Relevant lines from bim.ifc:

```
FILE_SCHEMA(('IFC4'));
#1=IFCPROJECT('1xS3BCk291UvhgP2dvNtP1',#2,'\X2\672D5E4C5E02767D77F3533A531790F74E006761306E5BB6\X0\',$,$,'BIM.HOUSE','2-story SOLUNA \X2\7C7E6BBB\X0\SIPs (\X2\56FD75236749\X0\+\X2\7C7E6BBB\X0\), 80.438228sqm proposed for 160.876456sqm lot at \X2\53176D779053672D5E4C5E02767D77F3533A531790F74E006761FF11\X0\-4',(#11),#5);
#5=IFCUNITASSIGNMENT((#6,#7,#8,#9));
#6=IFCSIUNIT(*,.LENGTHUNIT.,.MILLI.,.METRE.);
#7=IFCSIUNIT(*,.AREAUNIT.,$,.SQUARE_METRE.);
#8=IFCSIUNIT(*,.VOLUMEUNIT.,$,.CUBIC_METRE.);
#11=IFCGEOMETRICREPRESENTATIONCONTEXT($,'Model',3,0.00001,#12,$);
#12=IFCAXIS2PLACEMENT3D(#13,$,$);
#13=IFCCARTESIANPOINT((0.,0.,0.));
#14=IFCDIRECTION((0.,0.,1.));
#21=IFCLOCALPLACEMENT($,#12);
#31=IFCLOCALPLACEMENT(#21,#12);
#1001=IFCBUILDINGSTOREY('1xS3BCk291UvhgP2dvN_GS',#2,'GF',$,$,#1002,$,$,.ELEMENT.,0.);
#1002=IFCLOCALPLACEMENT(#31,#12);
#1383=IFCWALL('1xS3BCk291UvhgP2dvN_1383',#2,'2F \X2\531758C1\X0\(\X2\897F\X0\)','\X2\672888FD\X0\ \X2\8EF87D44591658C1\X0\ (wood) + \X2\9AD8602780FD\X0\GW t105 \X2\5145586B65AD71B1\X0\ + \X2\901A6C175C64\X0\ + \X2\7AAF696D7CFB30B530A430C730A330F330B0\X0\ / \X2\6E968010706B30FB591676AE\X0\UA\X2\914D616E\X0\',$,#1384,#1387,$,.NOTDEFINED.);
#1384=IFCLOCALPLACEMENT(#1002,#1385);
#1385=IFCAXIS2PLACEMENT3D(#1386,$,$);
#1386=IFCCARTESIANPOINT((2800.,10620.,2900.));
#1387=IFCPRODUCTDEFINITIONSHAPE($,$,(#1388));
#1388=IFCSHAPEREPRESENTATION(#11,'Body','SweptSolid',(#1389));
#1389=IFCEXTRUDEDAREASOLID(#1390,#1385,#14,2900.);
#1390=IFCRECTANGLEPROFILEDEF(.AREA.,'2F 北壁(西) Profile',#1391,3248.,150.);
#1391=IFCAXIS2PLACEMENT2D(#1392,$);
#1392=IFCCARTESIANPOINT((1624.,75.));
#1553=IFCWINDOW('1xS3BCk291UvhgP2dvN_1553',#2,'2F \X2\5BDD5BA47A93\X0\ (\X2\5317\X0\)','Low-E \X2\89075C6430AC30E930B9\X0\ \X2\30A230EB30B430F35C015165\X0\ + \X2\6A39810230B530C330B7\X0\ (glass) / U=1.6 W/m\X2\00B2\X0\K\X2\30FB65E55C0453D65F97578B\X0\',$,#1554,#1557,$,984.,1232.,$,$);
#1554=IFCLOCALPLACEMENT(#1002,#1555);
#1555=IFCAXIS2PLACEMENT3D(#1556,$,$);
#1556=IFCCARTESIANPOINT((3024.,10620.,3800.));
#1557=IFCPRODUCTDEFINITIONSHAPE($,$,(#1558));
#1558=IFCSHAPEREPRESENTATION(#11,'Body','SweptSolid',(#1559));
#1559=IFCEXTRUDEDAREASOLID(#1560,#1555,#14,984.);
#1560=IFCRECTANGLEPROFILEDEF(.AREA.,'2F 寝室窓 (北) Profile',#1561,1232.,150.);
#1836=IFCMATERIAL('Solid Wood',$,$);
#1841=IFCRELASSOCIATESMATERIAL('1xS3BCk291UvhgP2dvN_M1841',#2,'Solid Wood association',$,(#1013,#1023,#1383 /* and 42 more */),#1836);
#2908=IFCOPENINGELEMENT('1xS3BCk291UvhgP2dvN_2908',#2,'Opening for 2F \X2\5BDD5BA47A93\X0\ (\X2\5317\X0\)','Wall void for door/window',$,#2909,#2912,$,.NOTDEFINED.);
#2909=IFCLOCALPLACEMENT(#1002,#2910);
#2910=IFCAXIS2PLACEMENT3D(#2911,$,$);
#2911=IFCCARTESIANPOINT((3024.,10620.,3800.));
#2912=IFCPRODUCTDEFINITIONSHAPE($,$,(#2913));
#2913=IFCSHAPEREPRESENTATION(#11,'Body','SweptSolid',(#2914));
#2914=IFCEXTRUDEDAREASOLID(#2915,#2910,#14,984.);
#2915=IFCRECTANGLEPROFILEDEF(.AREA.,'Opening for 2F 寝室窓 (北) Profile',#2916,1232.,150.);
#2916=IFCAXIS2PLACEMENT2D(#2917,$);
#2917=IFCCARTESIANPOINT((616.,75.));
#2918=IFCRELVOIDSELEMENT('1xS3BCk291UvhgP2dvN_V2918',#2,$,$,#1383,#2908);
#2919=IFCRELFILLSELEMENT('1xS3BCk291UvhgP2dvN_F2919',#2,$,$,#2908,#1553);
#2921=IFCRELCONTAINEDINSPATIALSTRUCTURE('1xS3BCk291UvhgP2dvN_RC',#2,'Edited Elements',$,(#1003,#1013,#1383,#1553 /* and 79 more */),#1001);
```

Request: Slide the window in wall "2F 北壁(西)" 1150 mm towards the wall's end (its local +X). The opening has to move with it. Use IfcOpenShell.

```python
import ifcopenshell
import ifcopenshell.api.geometry
import ifcopenshell.util.placement

model = ifcopenshell.open("bim.ifc")

window = model.by_guid("1xS3BCk291UvhgP2dvN_1553")
opening = window.FillsVoids[0].RelatingOpeningElement
wall = opening.VoidsElements[0].RelatingBuildingElement

wall_matrix = ifcopenshell.util.placement.get_local_placement(wall.ObjectPlacement)
shift = wall_matrix[:3, 0] * 1150.0
before = ifcopenshell.util.placement.get_local_placement(window.ObjectPlacement)[:3, 3].copy()

# The window is not placed relative to its opening, so move both.
for product in (opening, window):
    matrix = ifcopenshell.util.placement.get_local_placement(product.ObjectPlacement)
    matrix[:3, 3] += shift
    ifcopenshell.api.geometry.edit_object_placement(model, product=product, matrix=matrix, is_si=False)

after = ifcopenshell.util.placement.get_local_placement(window.ObjectPlacement)[:3, 3]
print("window moved by", (after - before).round(3) + 0.0)

model.write("bim_rev.ifc")
```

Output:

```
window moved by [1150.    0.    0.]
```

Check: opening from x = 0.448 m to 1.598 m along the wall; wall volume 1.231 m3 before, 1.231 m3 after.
